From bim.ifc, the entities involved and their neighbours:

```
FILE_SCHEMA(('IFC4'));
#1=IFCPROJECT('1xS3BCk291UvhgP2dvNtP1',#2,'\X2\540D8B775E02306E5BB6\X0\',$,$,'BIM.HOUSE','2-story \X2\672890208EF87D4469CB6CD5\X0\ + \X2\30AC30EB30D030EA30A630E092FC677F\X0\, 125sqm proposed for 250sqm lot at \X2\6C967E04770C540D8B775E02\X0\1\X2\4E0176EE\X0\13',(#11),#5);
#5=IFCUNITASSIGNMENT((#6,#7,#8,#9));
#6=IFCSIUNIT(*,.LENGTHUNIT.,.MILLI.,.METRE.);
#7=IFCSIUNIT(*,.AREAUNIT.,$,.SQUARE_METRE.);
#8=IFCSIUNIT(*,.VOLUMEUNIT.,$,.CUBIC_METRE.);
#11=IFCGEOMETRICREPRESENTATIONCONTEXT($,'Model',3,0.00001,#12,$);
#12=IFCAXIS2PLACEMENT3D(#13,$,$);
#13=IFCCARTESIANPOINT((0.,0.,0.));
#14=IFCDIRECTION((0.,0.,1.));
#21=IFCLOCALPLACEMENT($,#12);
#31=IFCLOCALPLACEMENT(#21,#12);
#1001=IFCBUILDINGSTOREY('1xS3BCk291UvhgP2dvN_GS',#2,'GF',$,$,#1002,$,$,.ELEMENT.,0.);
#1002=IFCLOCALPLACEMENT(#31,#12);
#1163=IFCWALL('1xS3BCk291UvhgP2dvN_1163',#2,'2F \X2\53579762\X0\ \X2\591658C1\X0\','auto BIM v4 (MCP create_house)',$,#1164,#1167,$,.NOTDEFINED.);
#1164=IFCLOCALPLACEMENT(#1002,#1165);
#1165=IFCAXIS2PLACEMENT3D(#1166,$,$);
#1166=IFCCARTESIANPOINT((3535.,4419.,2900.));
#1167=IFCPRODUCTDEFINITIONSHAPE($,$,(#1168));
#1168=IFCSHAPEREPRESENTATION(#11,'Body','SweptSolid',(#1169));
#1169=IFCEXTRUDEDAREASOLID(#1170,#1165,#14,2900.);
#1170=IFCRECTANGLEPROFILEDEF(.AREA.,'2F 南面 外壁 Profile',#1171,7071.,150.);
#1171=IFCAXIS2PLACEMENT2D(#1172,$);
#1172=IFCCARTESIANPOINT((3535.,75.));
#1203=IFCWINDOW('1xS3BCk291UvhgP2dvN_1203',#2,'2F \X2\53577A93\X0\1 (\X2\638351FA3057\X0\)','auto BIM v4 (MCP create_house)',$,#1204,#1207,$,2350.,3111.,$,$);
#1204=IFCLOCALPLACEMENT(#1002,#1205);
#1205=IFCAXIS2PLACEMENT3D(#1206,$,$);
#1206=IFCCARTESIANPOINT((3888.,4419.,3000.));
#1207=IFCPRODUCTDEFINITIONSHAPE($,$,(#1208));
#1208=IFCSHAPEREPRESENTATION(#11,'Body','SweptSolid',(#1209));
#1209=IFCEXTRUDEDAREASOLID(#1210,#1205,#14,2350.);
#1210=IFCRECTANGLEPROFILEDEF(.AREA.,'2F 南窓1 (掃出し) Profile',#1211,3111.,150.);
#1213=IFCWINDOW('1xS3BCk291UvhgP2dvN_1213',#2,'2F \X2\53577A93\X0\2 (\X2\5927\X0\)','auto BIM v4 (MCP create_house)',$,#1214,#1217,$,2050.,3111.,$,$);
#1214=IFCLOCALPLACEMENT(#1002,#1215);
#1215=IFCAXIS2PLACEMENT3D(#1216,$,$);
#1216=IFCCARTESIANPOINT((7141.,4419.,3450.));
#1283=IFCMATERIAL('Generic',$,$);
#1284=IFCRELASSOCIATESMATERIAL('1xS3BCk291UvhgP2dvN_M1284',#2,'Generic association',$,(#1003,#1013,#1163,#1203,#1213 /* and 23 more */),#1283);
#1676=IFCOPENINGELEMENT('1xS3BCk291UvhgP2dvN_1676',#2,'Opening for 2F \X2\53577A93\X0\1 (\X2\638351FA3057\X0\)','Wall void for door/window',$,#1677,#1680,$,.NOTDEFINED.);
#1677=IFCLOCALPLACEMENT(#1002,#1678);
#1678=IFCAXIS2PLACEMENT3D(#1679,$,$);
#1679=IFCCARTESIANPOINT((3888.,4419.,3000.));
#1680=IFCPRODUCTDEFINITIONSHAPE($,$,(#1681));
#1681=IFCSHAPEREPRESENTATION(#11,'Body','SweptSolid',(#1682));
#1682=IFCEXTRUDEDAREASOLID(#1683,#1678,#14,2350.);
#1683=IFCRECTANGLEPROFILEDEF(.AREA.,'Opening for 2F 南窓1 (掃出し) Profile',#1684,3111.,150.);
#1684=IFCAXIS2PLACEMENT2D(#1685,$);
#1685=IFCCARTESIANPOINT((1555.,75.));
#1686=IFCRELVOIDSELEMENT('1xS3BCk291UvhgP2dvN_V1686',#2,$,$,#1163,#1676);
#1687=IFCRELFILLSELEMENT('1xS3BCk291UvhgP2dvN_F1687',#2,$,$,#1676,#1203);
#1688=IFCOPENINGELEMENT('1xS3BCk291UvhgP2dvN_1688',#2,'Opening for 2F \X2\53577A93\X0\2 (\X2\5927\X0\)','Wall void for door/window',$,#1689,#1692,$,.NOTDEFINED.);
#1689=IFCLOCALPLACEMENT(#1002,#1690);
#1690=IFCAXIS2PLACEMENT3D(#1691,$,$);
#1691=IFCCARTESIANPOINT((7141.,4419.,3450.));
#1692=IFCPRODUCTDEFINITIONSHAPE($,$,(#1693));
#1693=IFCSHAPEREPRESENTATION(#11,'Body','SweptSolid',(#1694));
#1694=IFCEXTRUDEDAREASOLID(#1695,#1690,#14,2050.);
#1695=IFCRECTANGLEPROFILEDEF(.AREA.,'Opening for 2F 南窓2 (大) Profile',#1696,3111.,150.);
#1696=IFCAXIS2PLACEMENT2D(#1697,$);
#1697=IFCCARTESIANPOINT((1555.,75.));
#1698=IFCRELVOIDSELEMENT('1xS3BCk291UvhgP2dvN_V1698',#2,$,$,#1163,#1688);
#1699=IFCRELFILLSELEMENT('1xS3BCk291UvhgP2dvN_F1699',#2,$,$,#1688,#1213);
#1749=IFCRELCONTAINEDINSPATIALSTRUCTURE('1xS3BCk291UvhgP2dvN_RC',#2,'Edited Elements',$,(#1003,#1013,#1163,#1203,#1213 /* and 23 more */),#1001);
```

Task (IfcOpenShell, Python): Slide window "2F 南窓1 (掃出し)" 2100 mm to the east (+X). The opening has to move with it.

```python
import ifcopenshell
import ifcopenshell.api.geometry
import ifcopenshell.util.placement

model = ifcopenshell.open("bim.ifc")

window = model.by_id(1203)
opening = window.FillsVoids[0].RelatingOpeningElement
wall = opening.VoidsElements[0].RelatingBuildingElement

wall_matrix = ifcopenshell.util.placement.get_local_placement(wall.ObjectPlacement)
shift = wall_matrix[:3, 0] * 2100.0
before = ifcopenshell.util.placement.get_local_placement(window.ObjectPlacement)[:3, 3].copy()

# The window is not placed relative to its opening, so move both.
for product in (opening, window):
    matrix = ifcopenshell.util.placement.get_local_placement(product.ObjectPlacement)
    matrix[:3, 3] += shift
    ifcopenshell.api.geometry.edit_object_placement(model, product=product, matrix=matrix, is_si=False)

after = ifcopenshell.util.placement.get_local_placement(window.ObjectPlacement)[:3, 3]
print("window moved by", (after - before).round(3) + 0.0)

model.write("bim_updated.ifc")
```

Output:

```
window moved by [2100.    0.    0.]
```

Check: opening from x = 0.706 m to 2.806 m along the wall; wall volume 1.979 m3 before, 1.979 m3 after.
